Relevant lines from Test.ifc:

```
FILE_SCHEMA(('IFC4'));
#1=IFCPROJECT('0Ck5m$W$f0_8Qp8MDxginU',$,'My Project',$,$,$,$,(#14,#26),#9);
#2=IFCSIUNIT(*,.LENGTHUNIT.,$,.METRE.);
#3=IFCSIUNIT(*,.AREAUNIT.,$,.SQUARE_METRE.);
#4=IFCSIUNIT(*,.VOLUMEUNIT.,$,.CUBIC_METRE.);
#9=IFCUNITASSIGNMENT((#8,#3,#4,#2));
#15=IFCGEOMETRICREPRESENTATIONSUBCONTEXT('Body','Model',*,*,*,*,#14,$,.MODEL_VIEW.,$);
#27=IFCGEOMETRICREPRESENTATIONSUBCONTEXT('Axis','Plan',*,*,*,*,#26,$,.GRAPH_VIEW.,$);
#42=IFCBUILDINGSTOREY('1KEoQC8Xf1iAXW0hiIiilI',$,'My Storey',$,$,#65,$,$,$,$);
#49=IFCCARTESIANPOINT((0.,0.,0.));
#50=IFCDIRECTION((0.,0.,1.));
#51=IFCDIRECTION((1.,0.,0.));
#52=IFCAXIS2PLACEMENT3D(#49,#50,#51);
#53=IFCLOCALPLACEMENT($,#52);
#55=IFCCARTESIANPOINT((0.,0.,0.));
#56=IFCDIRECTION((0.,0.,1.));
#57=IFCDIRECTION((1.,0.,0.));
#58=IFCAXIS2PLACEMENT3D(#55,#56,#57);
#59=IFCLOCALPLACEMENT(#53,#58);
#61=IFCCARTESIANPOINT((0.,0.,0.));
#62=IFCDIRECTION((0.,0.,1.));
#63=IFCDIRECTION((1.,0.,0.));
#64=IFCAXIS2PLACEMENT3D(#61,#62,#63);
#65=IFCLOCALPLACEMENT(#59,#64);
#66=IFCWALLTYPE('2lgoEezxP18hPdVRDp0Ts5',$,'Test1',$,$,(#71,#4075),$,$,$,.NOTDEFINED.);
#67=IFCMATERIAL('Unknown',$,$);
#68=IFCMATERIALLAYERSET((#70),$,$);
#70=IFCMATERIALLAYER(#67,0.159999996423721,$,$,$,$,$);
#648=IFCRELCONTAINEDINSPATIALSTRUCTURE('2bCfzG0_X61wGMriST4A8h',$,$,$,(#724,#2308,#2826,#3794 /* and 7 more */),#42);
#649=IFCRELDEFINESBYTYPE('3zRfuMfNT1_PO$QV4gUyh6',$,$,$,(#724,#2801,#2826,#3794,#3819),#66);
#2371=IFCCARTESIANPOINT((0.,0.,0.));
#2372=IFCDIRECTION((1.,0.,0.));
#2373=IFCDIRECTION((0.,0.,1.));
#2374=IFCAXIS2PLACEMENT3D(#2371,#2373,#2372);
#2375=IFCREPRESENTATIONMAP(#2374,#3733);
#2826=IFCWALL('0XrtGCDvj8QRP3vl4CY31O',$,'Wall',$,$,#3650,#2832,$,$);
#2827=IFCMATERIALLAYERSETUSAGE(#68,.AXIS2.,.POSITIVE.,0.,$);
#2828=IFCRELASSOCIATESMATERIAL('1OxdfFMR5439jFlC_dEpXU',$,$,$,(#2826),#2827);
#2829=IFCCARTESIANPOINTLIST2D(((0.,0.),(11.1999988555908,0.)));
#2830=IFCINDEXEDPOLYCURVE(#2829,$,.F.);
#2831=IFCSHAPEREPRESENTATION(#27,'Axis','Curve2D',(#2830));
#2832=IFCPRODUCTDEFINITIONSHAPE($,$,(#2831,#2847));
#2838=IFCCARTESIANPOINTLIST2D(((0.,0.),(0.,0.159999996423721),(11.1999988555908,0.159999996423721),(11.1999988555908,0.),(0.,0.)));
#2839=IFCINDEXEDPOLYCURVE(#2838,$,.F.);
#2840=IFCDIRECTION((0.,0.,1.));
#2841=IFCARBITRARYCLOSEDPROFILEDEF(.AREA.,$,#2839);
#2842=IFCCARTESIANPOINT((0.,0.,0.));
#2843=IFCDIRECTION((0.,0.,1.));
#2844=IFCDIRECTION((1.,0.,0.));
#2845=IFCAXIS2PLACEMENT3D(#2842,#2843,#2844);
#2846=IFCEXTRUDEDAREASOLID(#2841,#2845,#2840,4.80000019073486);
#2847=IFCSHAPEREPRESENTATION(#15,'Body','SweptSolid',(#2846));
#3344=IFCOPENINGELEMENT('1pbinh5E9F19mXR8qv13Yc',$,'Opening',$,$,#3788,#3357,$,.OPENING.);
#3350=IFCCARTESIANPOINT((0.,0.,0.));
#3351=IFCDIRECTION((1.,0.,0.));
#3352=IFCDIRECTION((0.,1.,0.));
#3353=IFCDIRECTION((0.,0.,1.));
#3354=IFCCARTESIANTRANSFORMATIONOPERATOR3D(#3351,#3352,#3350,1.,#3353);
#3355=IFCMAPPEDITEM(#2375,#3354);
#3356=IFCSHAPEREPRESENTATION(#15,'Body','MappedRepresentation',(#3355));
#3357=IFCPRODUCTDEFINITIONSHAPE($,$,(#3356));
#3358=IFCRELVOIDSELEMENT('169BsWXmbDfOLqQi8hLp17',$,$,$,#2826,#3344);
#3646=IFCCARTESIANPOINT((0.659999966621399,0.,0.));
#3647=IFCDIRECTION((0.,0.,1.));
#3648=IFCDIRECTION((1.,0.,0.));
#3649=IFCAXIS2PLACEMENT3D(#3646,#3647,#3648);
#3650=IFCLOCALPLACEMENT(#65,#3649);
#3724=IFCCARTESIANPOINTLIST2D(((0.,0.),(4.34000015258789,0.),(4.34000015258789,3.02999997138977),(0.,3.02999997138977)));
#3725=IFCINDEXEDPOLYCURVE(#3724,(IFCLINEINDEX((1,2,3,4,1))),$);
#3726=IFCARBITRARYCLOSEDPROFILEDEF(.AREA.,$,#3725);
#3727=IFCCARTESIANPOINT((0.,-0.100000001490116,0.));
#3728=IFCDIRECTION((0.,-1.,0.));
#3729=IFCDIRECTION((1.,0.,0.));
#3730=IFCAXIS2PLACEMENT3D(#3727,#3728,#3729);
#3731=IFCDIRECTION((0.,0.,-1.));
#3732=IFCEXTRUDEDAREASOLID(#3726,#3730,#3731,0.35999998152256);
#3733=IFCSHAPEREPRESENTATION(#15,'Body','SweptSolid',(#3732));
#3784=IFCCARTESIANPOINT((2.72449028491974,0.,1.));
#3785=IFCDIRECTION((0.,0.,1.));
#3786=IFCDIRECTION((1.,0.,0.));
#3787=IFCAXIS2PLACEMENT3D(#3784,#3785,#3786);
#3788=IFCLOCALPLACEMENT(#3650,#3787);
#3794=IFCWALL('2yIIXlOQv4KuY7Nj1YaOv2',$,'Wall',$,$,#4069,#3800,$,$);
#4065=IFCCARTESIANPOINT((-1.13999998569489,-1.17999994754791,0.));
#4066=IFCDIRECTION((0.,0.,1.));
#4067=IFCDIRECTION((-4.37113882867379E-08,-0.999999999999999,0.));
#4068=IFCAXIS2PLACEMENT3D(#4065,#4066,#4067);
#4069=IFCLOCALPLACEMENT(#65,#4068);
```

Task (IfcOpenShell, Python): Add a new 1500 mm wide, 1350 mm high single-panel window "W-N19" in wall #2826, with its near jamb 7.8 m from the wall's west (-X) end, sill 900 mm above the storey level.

```python
import numpy as np
import ifcopenshell
import ifcopenshell.api.feature
import ifcopenshell.api.geometry
import ifcopenshell.api.root
import ifcopenshell.api.spatial
import ifcopenshell.geom
import ifcopenshell.util.element
import ifcopenshell.util.placement
import ifcopenshell.util.representation
import ifcopenshell.util.shape
import ifcopenshell.util.unit

model = ifcopenshell.open("Test.ifc")
unit_scale = ifcopenshell.util.unit.calculate_unit_scale(model)
settings = ifcopenshell.geom.settings()


def volume(element):
    """Net volume in cubic metres, openings subtracted."""
    shape = ifcopenshell.geom.create_shape(settings, element)
    return ifcopenshell.util.shape.get_volume(shape.geometry)


wall = model.by_guid("0XrtGCDvj8QRP3vl4CY31O")
storey = ifcopenshell.util.element.get_container(wall, ifc_class="IfcBuildingStorey")
context = ifcopenshell.util.representation.get_context(model, "Model", "Body", "MODEL_VIEW")
before = volume(wall)

width, height, from_end, sill = 1.5, 1.35, 7.8, 0.9  # metres

# The wall runs along its own X axis, and the end named is its -X end.
wall_shape = ifcopenshell.geom.create_shape(settings, wall)
x, y, z = ifcopenshell.util.shape.get_vertices(wall_shape.geometry).T
start = x.min() + from_end
face, thickness = float(y.min()), float(y.max() - y.min())
wall_matrix = ifcopenshell.util.placement.get_local_placement(wall.ObjectPlacement)
level = ifcopenshell.util.placement.get_local_placement(storey.ObjectPlacement)[2, 3]


def in_wall(x, y):
    """Placement at x, y metres in the wall's axes, at sill height."""
    matrix = wall_matrix.copy()
    matrix[:, 3] = wall_matrix @ np.array([x / unit_scale, y / unit_scale, 0.0, 1.0])
    matrix[2, 3] = level + sill / unit_scale
    return matrix


# Opening: a box that overshoots both wall faces by 50 mm.
opening = ifcopenshell.api.root.create_entity(model, ifc_class="IfcOpeningElement", predefined_type="OPENING")
box = ifcopenshell.api.geometry.add_wall_representation(
    model, context=context, length=width, height=height, thickness=thickness + 0.1
)
ifcopenshell.api.geometry.assign_representation(model, product=opening, representation=box)
ifcopenshell.api.geometry.edit_object_placement(model, product=opening, matrix=in_wall(start, face - 0.05), is_si=False)
ifcopenshell.api.feature.add_feature(model, feature=opening, element=wall)

window = ifcopenshell.api.root.create_entity(model, ifc_class="IfcWindow", name="W-N19", predefined_type="WINDOW")
window.OverallWidth, window.OverallHeight = width / unit_scale, height / unit_scale
window.PartitioningType = "SINGLE_PANEL"
body = ifcopenshell.api.geometry.add_window_representation(
    model,
    context=context,
    overall_width=window.OverallWidth,
    overall_height=window.OverallHeight,
    partition_type="SINGLE_PANEL",
)
ifcopenshell.api.geometry.assign_representation(model, product=window, representation=body)
ifcopenshell.api.spatial.assign_container(model, products=[window], relating_structure=storey)
ifcopenshell.api.feature.add_filling(model, opening=opening, element=window)

# Centre the window in the wall's thickness.
ifcopenshell.api.geometry.edit_object_placement(model, product=window, matrix=in_wall(start, face), is_si=False)
window_shape = ifcopenshell.geom.create_shape(settings, window)
depth = ifcopenshell.util.shape.get_vertices(window_shape.geometry)[:, 1]
offset = face + thickness / 2 - (depth.min() + depth.max()) / 2
ifcopenshell.api.geometry.edit_object_placement(model, product=window, matrix=in_wall(start, offset), is_si=False)

after = volume(wall)

print(f"wall volume {before:.3f} -> {after:.3f} m3")

model.write("Test_updated.ifc")
```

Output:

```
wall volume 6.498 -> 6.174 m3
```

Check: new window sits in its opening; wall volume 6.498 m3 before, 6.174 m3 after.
